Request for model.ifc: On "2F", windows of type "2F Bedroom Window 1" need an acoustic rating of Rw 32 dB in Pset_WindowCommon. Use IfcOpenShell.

First a look at what the model holds.

```python
import ifcopenshell
import ifcopenshell.util.element

model = ifcopenshell.open("model.ifc")
print(model.schema)
storey = next(s for s in model.by_type("IfcBuildingStorey") if s.Name == "2F")
windows = [e for e in ifcopenshell.util.element.get_decomposition(storey) if e.is_a("IfcWindow")]
seen = {}
for e in windows:
    element_type = ifcopenshell.util.element.get_type(e)
    key = (element_type.Name if element_type != e and element_type else None, ifcopenshell.util.element.get_pset(e, "Pset_WindowCommon", "AcousticRating"))
    seen[key] = seen.get(key, 0) + 1
for (name, value), count in sorted(seen.items(), key=str):
    print(count, "x", name, "|", value)
```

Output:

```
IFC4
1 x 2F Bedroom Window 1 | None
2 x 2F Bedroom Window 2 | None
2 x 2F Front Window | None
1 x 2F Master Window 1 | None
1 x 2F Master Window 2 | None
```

```python
import ifcopenshell
import ifcopenshell.api.pset
import ifcopenshell.util.element

model = ifcopenshell.open("model.ifc")

storey = next(s for s in model.by_type("IfcBuildingStorey") if s.Name == "2F")
windows = [e for e in ifcopenshell.util.element.get_decomposition(storey) if e.is_a("IfcWindow")]

count = 0
for e in windows:
    element_type = ifcopenshell.util.element.get_type(e)
    if element_type in (None, e) or element_type.Name != "2F Bedroom Window 1":
        continue
    # add_pset returns the element's existing set when there is one.
    pset = ifcopenshell.api.pset.add_pset(model, product=e, name="Pset_WindowCommon")
    ifcopenshell.api.pset.edit_pset(model, pset=pset, properties={"AcousticRating": "Rw 32 dB"})
    count += 1

print(count, "windows updated")

model.write("model_updated.ifc")
```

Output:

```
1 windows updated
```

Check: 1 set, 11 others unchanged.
